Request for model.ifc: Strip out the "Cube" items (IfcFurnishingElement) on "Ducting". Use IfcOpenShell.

First a look at what the model holds.

```python
import ifcopenshell
import ifcopenshell.util.element

model = ifcopenshell.open("model.ifc")
print(model.schema)
storey = next(s for s in model.by_type("IfcBuildingStorey") if s.Name == "Ducting")
furniture = [e for e in ifcopenshell.util.element.get_decomposition(storey) if e.is_a("IfcFurnishingElement")]
seen = {}
for e in furniture:
    element_type = ifcopenshell.util.element.get_type(e)
    name = element_type.Name if element_type not in (None, e) else None
    seen[name] = seen.get(name, 0) + 1
for name, count in sorted(seen.items(), key=str):
    print(count, "x", name)
```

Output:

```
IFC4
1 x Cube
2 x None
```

```python
import ifcopenshell
import ifcopenshell.api.root
import ifcopenshell.util.element

model = ifcopenshell.open("model.ifc")

storey = next(s for s in model.by_type("IfcBuildingStorey") if s.Name == "Ducting")
furniture = [e for e in ifcopenshell.util.element.get_decomposition(storey) if e.is_a("IfcFurnishingElement")]
targets = [e for e in furniture if (t := ifcopenshell.util.element.get_type(e)) not in (None, e) and t.Name == "Cube"]

for e in targets:
    ifcopenshell.api.root.remove_product(model, product=e)
print(len(targets), "removed")

model.write("model_rev.ifc")
```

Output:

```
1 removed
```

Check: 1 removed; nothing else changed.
